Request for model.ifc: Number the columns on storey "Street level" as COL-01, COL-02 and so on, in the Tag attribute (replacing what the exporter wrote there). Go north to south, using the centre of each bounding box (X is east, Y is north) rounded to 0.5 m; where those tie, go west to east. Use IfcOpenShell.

First a look at what the model holds.

```python
import ifcopenshell
import ifcopenshell.util.element
import ifcopenshell.util.placement

model = ifcopenshell.open("model.ifc")
print(model.schema)
storey = next(s for s in model.by_type("IfcBuildingStorey") if s.Name == "Street level")
columns = [e for e in ifcopenshell.util.element.get_decomposition(storey) if e.is_a("IfcColumn")]
for e in sorted(columns, key=lambda e: e.id()):
    origin = ifcopenshell.util.placement.get_local_placement(e.ObjectPlacement)[:3, 3]
    print(e.id(), e.Tag, e.Name, origin.round(2) + 0.0, sep=" | ")
```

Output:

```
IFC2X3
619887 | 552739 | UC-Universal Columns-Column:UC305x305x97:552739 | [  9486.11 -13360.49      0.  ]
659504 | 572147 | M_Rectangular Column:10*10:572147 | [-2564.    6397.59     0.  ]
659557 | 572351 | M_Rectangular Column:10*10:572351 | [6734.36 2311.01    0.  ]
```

```python
import ifcopenshell
import ifcopenshell.geom
import ifcopenshell.util.element
import ifcopenshell.util.shape

model = ifcopenshell.open("model.ifc")
settings = ifcopenshell.geom.settings()
settings.set("use-world-coords", True)


def centre(element):
    shape = ifcopenshell.geom.create_shape(settings, element)
    return ifcopenshell.util.shape.get_bbox_centroid(shape.geometry)


storey = next(s for s in model.by_type("IfcBuildingStorey") if s.Name == "Street level")
columns = [e for e in ifcopenshell.util.element.get_decomposition(storey) if e.is_a("IfcColumn")]

# Insertion points can sit at a corner or the storey origin, so sort by the geometry (in metres).
centres = {e: centre(e) for e in columns}
columns.sort(key=lambda e: (-round(centres[e][1] / 0.5), centres[e][0]))

for i, e in enumerate(columns, start=1):
    number = f"COL-{i:02d}"
    e.Tag = number
    print(e.id(), number)

model.write("model_v2.ifc")
```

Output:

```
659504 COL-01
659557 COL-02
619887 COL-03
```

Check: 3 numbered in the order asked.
